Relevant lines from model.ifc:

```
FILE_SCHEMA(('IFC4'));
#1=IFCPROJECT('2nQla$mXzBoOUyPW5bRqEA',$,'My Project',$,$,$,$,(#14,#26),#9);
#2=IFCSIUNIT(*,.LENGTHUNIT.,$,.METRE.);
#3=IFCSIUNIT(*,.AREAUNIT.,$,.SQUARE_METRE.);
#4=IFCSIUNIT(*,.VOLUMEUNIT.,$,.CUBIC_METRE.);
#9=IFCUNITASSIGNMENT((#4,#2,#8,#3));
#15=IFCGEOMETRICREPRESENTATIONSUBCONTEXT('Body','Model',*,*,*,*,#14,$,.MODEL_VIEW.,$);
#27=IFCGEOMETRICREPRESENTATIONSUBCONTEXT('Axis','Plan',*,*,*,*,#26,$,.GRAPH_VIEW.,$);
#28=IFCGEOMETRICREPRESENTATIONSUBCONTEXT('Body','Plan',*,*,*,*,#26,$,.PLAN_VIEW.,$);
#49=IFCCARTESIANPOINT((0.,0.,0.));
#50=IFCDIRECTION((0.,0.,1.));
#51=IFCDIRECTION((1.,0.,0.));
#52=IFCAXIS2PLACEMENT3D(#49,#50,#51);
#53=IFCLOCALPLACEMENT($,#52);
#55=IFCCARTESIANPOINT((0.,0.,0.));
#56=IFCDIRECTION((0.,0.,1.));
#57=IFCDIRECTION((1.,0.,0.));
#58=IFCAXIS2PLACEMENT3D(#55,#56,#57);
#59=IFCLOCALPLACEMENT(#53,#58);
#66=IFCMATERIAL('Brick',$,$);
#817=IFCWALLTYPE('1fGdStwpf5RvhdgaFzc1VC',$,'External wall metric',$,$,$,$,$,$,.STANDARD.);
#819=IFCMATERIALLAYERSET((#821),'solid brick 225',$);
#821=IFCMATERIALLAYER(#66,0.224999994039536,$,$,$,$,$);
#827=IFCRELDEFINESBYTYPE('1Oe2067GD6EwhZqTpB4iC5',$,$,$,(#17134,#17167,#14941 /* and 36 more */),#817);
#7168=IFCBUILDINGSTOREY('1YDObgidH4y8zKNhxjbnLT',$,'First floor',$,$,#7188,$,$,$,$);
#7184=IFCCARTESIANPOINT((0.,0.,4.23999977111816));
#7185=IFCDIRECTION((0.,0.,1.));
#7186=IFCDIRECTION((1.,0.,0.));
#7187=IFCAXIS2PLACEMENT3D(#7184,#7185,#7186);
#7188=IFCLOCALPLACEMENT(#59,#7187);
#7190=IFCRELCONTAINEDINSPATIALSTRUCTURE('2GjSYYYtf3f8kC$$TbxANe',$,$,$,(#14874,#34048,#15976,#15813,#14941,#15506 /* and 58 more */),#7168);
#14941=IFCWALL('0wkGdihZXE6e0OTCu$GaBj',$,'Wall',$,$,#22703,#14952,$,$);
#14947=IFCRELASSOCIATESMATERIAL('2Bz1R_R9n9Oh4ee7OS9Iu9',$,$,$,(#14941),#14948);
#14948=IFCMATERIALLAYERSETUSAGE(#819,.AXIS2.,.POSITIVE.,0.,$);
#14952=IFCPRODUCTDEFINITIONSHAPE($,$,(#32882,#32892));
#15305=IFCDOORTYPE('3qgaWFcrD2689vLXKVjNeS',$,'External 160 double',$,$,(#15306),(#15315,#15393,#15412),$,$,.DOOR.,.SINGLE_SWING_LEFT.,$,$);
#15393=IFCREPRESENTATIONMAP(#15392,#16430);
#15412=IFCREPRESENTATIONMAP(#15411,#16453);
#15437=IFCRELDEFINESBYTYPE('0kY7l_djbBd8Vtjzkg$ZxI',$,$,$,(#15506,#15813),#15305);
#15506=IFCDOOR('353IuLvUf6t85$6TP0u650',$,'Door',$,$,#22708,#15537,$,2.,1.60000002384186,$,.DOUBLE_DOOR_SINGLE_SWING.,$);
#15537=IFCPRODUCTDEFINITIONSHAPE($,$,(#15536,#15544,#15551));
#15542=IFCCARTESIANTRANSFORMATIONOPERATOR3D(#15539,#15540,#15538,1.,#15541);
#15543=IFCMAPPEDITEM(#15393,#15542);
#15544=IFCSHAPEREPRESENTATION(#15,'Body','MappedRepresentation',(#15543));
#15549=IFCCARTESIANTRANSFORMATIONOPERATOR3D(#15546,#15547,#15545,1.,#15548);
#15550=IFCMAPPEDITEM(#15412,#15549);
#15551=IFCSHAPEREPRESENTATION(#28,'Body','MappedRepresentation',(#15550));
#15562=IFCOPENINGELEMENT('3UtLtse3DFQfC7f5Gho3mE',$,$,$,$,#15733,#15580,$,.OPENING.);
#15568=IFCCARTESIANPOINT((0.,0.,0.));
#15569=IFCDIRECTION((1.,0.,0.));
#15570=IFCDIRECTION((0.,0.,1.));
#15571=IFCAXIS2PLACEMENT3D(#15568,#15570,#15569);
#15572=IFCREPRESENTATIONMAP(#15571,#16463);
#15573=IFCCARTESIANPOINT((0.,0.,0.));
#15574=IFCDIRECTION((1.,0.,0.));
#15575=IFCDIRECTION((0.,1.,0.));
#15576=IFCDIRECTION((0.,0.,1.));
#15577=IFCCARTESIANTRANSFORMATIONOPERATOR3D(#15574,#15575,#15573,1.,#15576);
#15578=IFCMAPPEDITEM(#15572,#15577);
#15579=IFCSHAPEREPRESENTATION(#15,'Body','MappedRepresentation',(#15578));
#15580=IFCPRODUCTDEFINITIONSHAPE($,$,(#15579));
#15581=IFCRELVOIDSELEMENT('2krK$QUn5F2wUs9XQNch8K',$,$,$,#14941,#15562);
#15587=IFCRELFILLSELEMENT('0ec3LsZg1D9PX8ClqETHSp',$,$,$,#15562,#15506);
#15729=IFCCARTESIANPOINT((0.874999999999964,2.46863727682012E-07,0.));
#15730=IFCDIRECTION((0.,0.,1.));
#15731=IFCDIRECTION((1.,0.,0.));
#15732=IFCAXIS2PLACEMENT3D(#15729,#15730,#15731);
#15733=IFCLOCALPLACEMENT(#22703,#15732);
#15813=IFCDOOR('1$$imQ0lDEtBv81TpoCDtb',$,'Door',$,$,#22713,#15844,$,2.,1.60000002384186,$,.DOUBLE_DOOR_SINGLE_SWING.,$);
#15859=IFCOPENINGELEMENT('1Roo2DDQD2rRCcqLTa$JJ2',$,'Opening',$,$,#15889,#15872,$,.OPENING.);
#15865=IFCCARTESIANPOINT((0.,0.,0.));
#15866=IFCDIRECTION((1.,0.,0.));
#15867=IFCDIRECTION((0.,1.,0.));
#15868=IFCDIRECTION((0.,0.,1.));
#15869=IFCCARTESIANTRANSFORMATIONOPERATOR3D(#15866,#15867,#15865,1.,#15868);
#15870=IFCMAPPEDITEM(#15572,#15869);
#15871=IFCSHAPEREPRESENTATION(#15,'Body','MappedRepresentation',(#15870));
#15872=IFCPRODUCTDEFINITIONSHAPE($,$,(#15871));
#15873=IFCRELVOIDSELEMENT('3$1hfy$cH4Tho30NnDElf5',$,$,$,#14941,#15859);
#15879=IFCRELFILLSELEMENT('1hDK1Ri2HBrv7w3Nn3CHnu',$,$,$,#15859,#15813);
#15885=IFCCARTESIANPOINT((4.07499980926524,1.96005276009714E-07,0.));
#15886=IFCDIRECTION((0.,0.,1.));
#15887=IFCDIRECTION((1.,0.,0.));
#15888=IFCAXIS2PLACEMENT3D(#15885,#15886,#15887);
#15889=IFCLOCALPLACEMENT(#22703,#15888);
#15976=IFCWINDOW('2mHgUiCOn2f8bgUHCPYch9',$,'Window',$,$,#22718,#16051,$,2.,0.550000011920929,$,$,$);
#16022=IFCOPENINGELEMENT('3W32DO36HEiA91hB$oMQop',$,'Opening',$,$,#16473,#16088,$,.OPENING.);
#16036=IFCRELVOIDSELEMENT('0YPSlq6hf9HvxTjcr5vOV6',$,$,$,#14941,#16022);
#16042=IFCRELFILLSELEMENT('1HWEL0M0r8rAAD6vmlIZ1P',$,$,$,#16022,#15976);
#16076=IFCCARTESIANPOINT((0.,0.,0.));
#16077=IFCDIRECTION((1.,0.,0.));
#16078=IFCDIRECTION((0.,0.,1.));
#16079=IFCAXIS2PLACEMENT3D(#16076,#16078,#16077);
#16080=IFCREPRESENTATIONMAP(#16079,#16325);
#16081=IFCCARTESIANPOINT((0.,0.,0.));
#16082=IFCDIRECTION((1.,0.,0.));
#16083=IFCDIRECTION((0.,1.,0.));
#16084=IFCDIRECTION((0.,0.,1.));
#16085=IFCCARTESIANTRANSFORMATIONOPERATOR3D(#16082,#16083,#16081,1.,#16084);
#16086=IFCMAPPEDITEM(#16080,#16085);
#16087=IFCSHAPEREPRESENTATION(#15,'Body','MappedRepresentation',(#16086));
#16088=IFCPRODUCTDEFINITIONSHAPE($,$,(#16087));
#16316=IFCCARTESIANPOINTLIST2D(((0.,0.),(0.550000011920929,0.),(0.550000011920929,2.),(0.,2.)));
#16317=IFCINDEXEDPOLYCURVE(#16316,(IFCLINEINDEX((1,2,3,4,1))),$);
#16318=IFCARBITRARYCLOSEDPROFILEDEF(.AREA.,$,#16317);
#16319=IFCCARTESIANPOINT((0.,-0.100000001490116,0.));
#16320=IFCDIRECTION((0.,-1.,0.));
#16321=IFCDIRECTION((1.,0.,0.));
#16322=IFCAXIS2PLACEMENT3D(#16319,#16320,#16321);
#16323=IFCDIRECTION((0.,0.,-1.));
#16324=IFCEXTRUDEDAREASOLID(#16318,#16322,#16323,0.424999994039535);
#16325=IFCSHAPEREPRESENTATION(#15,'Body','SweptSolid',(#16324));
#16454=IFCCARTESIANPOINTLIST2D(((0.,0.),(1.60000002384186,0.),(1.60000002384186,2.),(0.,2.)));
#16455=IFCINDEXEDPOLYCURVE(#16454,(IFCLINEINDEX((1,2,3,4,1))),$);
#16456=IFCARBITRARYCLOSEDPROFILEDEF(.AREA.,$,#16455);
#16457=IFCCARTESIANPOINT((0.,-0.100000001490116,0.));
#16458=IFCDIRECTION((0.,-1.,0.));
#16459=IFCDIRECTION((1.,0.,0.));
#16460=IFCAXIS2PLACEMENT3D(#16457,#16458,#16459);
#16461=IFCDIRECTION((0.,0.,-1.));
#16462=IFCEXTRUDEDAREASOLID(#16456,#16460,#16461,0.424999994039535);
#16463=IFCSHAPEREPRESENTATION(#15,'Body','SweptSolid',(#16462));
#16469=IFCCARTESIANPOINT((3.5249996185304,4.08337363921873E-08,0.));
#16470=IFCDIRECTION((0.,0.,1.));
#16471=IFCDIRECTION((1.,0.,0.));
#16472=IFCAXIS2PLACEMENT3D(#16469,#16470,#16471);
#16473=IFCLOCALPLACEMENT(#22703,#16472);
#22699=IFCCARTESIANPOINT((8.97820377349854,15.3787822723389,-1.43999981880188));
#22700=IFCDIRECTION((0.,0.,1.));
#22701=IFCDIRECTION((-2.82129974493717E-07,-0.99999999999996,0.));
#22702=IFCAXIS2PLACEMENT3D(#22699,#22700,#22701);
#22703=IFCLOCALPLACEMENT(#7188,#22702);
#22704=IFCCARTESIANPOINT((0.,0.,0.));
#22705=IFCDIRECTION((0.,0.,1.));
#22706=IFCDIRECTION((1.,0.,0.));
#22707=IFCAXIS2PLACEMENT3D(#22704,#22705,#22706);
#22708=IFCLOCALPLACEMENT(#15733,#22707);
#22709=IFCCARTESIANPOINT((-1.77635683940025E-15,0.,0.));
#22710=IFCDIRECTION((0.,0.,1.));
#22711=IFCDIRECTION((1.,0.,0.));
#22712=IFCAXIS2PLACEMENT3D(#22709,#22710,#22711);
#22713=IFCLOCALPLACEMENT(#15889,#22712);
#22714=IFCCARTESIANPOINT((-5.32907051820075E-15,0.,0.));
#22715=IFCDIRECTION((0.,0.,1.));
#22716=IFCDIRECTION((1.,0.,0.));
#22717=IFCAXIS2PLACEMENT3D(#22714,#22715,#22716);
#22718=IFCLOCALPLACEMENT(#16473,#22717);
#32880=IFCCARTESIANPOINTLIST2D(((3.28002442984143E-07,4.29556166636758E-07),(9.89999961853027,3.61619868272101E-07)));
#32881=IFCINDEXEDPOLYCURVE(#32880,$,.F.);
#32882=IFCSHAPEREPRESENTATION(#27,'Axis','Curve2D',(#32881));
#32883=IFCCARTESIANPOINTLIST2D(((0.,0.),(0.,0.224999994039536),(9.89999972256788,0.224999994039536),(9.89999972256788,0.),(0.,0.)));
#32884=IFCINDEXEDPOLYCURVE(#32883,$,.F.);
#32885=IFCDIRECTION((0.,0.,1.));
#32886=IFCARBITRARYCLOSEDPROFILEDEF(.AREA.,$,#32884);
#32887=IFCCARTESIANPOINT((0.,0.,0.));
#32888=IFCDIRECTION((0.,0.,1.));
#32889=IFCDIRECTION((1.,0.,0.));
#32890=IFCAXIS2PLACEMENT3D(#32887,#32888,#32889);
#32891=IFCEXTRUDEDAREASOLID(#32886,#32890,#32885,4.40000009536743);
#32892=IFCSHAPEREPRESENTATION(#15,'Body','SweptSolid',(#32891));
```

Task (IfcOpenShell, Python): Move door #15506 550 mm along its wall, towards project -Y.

```python
import ifcopenshell
import ifcopenshell.api.geometry
import ifcopenshell.util.placement

model = ifcopenshell.open("model.ifc")

door = model.by_guid("353IuLvUf6t85$6TP0u650")
opening = door.FillsVoids[0].RelatingOpeningElement
wall = opening.VoidsElements[0].RelatingBuildingElement

wall_matrix = ifcopenshell.util.placement.get_local_placement(wall.ObjectPlacement)
shift = wall_matrix[:3, 0] * 0.55
before = ifcopenshell.util.placement.get_local_placement(door.ObjectPlacement)[:3, 3].copy()

# The door is placed relative to its opening, so it follows when the opening moves.
matrix = ifcopenshell.util.placement.get_local_placement(opening.ObjectPlacement)
matrix[:3, 3] += shift
ifcopenshell.api.geometry.edit_object_placement(
    model, product=opening, matrix=matrix, is_si=False, should_transform_children=True
)

after = ifcopenshell.util.placement.get_local_placement(door.ObjectPlacement)[:3, 3]
print("door moved by", (after - before).round(3) + 0.0)

model.write("model_rev.ifc")
```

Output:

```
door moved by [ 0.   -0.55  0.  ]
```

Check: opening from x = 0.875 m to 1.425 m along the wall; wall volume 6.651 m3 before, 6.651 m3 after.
